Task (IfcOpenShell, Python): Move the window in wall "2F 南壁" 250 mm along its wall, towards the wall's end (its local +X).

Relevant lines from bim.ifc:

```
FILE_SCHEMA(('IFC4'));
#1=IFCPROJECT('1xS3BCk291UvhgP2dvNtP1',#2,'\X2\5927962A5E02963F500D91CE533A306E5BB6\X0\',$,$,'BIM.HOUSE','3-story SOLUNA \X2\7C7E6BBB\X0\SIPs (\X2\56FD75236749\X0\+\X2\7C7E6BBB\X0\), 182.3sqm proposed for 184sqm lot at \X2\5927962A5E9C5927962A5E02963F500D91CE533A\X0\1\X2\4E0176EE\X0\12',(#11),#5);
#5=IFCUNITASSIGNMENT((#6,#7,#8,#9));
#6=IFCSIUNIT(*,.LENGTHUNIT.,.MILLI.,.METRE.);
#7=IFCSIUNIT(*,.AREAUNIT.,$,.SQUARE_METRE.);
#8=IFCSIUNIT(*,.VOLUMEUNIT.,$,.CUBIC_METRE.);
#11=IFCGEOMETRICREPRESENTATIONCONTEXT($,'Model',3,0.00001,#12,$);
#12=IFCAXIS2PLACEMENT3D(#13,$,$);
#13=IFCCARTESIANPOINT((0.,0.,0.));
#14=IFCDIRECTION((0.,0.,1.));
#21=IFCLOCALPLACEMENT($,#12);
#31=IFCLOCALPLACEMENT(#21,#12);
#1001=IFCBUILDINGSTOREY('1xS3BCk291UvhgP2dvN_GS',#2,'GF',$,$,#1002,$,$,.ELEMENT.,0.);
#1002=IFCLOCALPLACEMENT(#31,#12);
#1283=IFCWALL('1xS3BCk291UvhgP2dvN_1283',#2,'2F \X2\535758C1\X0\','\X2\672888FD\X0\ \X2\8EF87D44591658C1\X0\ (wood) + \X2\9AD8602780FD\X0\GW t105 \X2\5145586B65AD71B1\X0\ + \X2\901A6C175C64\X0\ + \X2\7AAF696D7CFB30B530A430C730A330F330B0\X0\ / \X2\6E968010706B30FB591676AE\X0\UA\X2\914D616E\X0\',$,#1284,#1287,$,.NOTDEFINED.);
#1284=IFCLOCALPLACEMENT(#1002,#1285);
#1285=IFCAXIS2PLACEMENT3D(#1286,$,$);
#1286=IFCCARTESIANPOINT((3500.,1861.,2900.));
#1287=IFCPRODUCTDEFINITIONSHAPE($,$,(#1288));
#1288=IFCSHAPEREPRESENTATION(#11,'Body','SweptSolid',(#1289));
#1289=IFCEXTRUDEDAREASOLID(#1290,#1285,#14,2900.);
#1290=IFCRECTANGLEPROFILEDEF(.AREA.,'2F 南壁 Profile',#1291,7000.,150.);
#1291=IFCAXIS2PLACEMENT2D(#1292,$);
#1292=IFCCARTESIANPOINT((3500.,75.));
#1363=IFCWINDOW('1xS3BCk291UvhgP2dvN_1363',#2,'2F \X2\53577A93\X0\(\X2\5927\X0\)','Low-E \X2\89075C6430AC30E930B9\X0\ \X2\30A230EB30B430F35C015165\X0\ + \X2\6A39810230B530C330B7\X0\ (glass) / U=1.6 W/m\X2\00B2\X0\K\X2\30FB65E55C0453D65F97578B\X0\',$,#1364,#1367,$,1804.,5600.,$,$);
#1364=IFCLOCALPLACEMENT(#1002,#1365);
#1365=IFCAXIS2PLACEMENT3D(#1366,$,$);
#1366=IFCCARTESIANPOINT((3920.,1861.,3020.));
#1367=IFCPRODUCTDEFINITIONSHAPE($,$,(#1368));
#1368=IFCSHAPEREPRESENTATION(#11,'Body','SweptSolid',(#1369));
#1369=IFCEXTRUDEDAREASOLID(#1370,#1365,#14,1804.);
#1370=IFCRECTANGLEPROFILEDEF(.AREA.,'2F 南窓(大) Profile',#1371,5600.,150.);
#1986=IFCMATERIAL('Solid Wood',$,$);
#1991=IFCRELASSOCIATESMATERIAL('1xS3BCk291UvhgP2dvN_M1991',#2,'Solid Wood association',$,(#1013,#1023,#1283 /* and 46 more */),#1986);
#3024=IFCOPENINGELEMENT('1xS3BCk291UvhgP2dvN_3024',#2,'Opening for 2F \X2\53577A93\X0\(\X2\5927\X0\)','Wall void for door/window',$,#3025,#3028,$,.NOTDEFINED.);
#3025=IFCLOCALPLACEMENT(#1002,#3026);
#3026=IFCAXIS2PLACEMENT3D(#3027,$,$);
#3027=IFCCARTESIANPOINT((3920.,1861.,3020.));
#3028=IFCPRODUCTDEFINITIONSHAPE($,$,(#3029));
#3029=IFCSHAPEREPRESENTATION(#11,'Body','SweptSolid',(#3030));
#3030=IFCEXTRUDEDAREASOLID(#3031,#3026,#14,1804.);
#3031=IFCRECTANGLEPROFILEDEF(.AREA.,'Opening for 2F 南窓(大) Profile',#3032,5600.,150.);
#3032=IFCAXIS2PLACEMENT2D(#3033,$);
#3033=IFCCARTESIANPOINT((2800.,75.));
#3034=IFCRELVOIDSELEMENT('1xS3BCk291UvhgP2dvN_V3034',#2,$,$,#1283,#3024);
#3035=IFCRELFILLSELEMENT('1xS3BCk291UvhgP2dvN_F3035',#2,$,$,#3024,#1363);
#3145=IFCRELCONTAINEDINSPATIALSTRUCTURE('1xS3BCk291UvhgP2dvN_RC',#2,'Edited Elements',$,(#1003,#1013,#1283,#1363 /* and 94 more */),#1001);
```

```python
import ifcopenshell
import ifcopenshell.api.geometry
import ifcopenshell.util.placement
import ifcopenshell.util.unit

model = ifcopenshell.open("bim.ifc")
unit_scale = ifcopenshell.util.unit.calculate_unit_scale(model)

window = model.by_id(1363)
opening = window.FillsVoids[0].RelatingOpeningElement
wall = opening.VoidsElements[0].RelatingBuildingElement

wall_matrix = ifcopenshell.util.placement.get_local_placement(wall.ObjectPlacement)
shift = wall_matrix[:3, 0] * 0.25 / unit_scale
before = ifcopenshell.util.placement.get_local_placement(window.ObjectPlacement)[:3, 3].copy()

# The window is not placed relative to its opening, so move both.
for product in (opening, window):
    matrix = ifcopenshell.util.placement.get_local_placement(product.ObjectPlacement)
    matrix[:3, 3] += shift
    ifcopenshell.api.geometry.edit_object_placement(model, product=product, matrix=matrix, is_si=False)

after = ifcopenshell.util.placement.get_local_placement(window.ObjectPlacement)[:3, 3]
print("window moved by", (after - before).round(3) + 0.0)

model.write("bim_edited.ifc")
```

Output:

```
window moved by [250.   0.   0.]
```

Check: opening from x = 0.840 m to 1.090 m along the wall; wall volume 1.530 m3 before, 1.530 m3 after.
